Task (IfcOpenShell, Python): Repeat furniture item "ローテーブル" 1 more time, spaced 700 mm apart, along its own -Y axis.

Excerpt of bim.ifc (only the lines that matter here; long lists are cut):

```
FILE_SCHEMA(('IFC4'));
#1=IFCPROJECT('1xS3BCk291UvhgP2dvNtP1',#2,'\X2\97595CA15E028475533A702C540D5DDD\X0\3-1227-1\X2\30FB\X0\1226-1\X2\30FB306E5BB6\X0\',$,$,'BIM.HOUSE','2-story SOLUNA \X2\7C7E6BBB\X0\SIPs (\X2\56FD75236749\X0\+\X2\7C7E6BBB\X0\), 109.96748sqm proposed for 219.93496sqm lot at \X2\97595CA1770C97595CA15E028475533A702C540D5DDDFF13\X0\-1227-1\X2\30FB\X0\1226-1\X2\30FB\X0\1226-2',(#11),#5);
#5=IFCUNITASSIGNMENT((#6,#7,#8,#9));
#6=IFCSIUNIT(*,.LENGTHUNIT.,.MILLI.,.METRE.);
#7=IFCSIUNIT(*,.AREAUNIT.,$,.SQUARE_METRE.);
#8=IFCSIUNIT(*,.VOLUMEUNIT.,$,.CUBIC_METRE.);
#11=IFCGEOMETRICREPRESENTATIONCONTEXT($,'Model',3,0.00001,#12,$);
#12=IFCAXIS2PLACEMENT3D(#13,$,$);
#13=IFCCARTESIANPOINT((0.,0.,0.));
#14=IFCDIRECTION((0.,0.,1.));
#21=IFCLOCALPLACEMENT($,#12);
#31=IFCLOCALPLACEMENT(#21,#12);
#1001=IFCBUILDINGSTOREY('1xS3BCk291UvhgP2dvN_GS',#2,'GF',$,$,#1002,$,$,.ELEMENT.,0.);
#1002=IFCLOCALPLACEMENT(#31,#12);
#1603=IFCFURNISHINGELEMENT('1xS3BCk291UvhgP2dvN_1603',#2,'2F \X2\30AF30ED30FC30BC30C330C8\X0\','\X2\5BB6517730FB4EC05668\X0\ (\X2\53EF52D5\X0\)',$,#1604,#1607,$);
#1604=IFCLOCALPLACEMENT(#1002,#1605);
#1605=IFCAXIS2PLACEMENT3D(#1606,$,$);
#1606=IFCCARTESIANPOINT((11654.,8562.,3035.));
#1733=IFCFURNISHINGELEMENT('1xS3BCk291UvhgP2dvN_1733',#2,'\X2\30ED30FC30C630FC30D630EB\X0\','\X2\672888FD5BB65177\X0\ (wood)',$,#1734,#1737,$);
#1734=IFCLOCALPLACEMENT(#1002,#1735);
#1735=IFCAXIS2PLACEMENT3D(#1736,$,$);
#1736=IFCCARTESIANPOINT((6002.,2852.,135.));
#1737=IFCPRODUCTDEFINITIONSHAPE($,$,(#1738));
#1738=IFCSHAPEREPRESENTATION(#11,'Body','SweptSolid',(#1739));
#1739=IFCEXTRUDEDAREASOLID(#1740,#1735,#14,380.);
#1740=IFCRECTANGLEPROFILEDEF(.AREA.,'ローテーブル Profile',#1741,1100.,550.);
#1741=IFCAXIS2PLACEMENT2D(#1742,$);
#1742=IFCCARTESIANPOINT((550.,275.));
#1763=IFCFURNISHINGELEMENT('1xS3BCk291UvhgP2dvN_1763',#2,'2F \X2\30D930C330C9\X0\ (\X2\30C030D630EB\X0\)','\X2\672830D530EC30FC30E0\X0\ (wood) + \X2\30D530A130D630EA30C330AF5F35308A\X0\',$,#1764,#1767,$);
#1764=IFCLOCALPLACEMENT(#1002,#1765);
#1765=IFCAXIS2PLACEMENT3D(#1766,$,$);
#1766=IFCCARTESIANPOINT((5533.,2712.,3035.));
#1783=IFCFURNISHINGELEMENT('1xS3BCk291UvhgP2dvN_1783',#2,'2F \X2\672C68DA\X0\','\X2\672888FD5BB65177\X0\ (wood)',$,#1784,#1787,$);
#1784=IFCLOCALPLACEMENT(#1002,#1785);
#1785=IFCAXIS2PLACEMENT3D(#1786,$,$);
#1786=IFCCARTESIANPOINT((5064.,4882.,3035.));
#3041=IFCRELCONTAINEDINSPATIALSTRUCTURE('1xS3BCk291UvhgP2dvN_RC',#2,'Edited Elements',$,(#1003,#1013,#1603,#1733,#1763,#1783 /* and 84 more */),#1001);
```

```python
import ifcopenshell
import ifcopenshell.api.geometry
import ifcopenshell.api.root
import ifcopenshell.util.element
import ifcopenshell.util.placement

model = ifcopenshell.open("bim.ifc")


def reuse_history(source, copy):
    """copy_class also copies each property set's owner history, people and application; keep the originals."""
    for rel in copy.IsDefinedBy:
        if rel.is_a("IfcRelDefinesByProperties") and (history := rel.RelatingPropertyDefinition.OwnerHistory):
            rel.RelatingPropertyDefinition.OwnerHistory = source.OwnerHistory
            ifcopenshell.util.element.remove_deep2(model, history)


source = model.by_guid("1xS3BCk291UvhgP2dvN_1733")
base = ifcopenshell.util.placement.get_local_placement(source.ObjectPlacement)
step = -base[:3, 1] * 700.0

for i in range(1, 2):
    copy = ifcopenshell.api.root.copy_class(model, product=source)
    copy.Representation = ifcopenshell.util.element.copy_deep(
        model, source.Representation, exclude=["IfcGeometricRepresentationContext", "IfcRepresentationMap"]
    )
    reuse_history(source, copy)
    matrix = base.copy()
    matrix[:3, 3] += i * step
    print("added at", matrix[:3, 3].round(3) + 0.0)
    ifcopenshell.api.geometry.edit_object_placement(model, product=copy, matrix=matrix, is_si=False)

model.write("bim_updated.ifc")
```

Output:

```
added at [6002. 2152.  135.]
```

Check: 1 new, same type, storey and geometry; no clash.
